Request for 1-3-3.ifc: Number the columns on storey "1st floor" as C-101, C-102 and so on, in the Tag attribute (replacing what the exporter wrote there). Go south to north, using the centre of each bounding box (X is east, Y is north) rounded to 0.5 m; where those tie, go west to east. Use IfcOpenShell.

First a look at what the model holds.

```python
import ifcopenshell
import ifcopenshell.util.element
import ifcopenshell.util.placement

model = ifcopenshell.open("1-3-3.ifc")
print(model.schema)
storey = next(s for s in model.by_type("IfcBuildingStorey") if s.Name == "1st floor")
columns = [e for e in ifcopenshell.util.element.get_decomposition(storey) if e.is_a("IfcColumn")]
for e in sorted(columns, key=lambda e: e.id()):
    origin = ifcopenshell.util.placement.get_local_placement(e.ObjectPlacement)[:3, 3]
    print(e.id(), e.Tag, e.Name, origin.round(2) + 0.0, sep=" | ")
```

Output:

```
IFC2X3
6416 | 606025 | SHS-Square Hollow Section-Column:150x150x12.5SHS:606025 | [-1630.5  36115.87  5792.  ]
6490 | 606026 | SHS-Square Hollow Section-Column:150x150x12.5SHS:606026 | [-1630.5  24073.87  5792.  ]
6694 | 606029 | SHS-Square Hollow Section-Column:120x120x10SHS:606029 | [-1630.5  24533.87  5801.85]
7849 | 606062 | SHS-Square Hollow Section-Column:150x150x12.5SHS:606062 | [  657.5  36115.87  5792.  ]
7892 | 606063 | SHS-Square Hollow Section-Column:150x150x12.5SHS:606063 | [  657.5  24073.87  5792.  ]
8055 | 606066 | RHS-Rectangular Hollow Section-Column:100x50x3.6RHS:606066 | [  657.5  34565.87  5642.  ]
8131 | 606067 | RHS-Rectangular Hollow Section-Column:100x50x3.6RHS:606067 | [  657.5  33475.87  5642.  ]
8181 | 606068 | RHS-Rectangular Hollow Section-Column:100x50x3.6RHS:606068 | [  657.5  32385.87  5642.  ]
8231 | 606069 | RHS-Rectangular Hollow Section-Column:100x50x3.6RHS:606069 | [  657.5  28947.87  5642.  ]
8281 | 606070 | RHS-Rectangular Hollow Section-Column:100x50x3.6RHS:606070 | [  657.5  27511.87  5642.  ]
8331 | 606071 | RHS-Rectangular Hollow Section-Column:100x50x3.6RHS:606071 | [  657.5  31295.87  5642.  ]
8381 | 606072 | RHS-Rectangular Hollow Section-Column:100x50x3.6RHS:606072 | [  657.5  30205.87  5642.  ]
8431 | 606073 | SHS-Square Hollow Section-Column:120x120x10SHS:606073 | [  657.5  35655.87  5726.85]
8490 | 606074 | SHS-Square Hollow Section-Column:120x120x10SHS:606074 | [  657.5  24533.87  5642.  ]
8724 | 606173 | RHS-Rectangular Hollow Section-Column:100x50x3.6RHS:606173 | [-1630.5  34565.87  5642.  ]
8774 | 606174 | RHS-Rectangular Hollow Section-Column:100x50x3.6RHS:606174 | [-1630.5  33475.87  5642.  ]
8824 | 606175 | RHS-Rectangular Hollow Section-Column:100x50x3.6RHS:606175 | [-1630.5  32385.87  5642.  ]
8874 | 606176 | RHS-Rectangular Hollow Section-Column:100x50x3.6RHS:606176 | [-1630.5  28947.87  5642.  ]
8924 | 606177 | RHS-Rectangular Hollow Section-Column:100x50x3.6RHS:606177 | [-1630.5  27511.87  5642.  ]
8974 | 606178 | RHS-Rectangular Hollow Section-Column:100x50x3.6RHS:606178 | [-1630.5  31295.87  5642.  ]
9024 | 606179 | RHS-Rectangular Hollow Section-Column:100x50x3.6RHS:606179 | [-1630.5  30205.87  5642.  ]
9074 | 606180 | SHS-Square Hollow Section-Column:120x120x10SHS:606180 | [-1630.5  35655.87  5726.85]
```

```python
import ifcopenshell
import ifcopenshell.geom
import ifcopenshell.util.element
import ifcopenshell.util.shape

model = ifcopenshell.open("1-3-3.ifc")
settings = ifcopenshell.geom.settings()
settings.set("use-world-coords", True)


def centre(element):
    shape = ifcopenshell.geom.create_shape(settings, element)
    return ifcopenshell.util.shape.get_bbox_centroid(shape.geometry)


storey = next(s for s in model.by_type("IfcBuildingStorey") if s.Name == "1st floor")
columns = [e for e in ifcopenshell.util.element.get_decomposition(storey) if e.is_a("IfcColumn")]

# Insertion points can sit at a corner or the storey origin, so sort by the geometry (in metres).
centres = {e: centre(e) for e in columns}
columns.sort(key=lambda e: (round(centres[e][1] / 0.5), centres[e][0]))

for i, e in enumerate(columns, start=1):
    number = f"C-1{i:02d}"
    e.Tag = number
    print(e.id(), number)

model.write("1-3-3_edited.ifc")
```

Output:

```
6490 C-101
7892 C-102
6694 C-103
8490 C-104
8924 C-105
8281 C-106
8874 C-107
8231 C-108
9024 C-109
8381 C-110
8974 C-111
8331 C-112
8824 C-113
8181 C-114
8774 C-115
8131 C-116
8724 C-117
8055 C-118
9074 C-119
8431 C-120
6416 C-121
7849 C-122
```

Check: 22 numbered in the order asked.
